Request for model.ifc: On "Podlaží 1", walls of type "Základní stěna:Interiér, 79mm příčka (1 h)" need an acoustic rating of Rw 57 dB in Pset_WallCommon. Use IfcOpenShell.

First a look at what the model holds.

```python
import ifcopenshell
import ifcopenshell.util.element

model = ifcopenshell.open("model.ifc")
print(model.schema)
storey = next(s for s in model.by_type("IfcBuildingStorey") if s.Name == "Podlaží 1")
walls = [e for e in ifcopenshell.util.element.get_decomposition(storey) if e.is_a("IfcWall")]
seen = {}
for e in walls:
    element_type = ifcopenshell.util.element.get_type(e)
    key = (element_type.Name if element_type != e and element_type else None, ifcopenshell.util.element.get_pset(e, "Pset_WallCommon", "AcousticRating"))
    seen[key] = seen.get(key, 0) + 1
for (name, value), count in sorted(seen.items(), key=str):
    print(count, "x", name, "|", value)
```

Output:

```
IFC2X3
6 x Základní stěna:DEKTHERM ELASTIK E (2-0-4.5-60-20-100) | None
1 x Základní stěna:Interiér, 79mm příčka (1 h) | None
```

```python
import ifcopenshell
import ifcopenshell.api.pset
import ifcopenshell.util.element

model = ifcopenshell.open("model.ifc")

storey = next(s for s in model.by_type("IfcBuildingStorey") if s.Name == "Podlaží 1")
walls = [e for e in ifcopenshell.util.element.get_decomposition(storey) if e.is_a("IfcWall")]

count = 0
for e in walls:
    element_type = ifcopenshell.util.element.get_type(e)
    if element_type in (None, e) or element_type.Name != "Základní stěna:Interiér, 79mm příčka (1 h)":
        continue
    # add_pset returns the element's existing set when there is one.
    pset = ifcopenshell.api.pset.add_pset(model, product=e, name="Pset_WallCommon")
    ifcopenshell.api.pset.edit_pset(model, pset=pset, properties={"AcousticRating": "Rw 57 dB"})
    count += 1

print(count, "walls updated")

model.write("model_updated.ifc")
```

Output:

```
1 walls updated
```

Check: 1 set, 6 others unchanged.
